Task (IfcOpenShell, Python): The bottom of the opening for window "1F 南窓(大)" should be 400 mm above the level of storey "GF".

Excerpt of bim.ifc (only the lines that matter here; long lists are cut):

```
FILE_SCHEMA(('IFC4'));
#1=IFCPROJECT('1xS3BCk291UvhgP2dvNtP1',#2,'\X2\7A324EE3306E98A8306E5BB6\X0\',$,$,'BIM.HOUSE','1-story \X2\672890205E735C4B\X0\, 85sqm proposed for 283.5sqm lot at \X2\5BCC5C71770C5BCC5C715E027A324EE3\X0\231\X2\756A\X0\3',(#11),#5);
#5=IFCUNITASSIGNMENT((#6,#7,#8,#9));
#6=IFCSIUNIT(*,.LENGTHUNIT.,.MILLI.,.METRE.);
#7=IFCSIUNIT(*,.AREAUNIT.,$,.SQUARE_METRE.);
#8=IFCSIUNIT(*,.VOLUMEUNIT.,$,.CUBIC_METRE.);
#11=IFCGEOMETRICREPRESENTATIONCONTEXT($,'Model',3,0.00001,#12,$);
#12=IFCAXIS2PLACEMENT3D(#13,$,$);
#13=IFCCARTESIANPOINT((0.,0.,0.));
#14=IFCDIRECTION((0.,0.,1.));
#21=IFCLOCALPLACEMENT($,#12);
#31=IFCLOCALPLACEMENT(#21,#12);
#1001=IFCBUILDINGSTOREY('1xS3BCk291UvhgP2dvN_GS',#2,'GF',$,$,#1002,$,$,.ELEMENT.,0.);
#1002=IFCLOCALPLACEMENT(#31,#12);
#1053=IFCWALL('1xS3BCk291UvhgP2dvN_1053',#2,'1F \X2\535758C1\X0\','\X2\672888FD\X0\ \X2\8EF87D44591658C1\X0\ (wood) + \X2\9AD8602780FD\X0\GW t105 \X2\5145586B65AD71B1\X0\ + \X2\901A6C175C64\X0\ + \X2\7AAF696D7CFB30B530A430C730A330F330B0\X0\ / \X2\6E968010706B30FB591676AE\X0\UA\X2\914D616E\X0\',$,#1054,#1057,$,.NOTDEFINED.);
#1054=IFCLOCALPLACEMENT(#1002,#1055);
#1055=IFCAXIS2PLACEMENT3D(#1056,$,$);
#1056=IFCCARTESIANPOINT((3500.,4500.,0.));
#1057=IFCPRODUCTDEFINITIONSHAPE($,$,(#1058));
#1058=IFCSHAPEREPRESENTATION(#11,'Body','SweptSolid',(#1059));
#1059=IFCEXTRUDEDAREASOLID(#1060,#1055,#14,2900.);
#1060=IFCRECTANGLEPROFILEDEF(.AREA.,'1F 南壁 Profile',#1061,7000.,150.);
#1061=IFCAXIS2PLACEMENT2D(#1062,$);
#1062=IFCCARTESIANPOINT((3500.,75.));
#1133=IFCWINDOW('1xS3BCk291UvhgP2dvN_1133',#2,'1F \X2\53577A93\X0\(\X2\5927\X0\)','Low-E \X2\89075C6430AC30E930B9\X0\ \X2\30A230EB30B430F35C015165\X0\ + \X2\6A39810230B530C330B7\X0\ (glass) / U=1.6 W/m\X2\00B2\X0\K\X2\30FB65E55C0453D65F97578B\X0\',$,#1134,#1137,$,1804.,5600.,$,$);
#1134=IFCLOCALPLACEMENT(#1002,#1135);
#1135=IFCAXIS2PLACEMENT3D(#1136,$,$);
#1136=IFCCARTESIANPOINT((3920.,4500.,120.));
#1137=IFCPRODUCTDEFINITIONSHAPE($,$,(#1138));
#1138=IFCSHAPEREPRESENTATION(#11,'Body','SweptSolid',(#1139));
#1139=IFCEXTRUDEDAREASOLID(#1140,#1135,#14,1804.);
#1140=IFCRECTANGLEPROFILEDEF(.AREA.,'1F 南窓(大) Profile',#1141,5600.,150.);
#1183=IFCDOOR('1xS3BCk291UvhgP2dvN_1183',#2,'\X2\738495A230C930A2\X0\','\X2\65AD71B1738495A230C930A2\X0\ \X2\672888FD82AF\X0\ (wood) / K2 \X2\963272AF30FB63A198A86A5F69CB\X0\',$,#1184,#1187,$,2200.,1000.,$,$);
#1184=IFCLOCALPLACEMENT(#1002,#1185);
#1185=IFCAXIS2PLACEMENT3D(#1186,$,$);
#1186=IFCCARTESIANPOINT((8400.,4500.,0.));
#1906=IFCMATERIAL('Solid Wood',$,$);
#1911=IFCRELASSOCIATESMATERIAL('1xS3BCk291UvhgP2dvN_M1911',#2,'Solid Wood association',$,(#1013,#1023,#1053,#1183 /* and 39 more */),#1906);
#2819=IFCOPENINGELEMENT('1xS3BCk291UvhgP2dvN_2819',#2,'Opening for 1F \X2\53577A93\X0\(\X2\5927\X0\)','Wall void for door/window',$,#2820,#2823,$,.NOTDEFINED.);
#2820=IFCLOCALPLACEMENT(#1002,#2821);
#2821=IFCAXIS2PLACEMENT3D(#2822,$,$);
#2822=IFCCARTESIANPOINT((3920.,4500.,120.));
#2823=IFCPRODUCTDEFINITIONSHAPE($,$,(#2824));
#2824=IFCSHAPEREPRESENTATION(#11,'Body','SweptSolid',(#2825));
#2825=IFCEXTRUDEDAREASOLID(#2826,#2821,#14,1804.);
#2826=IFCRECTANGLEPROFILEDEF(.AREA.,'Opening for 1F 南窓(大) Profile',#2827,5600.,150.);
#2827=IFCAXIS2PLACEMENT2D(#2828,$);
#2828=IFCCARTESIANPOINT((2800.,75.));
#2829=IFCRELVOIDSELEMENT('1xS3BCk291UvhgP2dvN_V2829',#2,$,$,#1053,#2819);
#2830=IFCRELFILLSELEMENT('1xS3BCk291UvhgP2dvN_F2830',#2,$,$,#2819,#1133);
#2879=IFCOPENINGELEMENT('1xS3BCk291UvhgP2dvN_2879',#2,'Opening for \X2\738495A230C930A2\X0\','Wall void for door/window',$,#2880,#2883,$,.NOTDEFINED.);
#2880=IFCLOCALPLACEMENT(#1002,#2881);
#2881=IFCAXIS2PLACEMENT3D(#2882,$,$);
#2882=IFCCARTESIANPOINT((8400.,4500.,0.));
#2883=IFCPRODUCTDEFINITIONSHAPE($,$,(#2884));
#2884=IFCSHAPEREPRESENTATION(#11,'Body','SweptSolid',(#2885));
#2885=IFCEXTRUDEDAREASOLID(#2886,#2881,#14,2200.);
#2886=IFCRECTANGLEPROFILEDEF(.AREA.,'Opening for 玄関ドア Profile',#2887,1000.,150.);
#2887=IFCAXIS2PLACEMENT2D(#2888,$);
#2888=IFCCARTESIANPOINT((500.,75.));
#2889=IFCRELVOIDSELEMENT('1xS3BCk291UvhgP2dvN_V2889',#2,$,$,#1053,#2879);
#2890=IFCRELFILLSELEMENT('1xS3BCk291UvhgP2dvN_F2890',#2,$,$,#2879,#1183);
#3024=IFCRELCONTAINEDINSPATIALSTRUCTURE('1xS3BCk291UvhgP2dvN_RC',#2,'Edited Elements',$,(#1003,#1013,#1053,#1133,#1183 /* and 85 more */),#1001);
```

```python
import numpy as np
import ifcopenshell
import ifcopenshell.api.geometry
import ifcopenshell.geom
import ifcopenshell.util.element
import ifcopenshell.util.placement
import ifcopenshell.util.shape
import ifcopenshell.util.unit

model = ifcopenshell.open("bim.ifc")
unit_scale = ifcopenshell.util.unit.calculate_unit_scale(model)

window = model.by_guid("1xS3BCk291UvhgP2dvN_1133")
opening = window.FillsVoids[0].RelatingOpeningElement
storey = ifcopenshell.util.element.get_container(window, ifc_class="IfcBuildingStorey")
level = ifcopenshell.util.placement.get_local_placement(storey.ObjectPlacement)[2, 3]

# The opening's origin need not be at the sill, so measure its lowest point.
shape = ifcopenshell.geom.create_shape(ifcopenshell.geom.settings(), opening)
bottom = ifcopenshell.util.shape.get_shape_bottom_elevation(shape, shape.geometry) / unit_scale
dz = level + 400.0 - bottom

shift = np.array([0.0, 0.0, dz])
# The window is not placed relative to its opening, so move both.
for product in (opening, window):
    matrix = ifcopenshell.util.placement.get_local_placement(product.ObjectPlacement)
    matrix[:3, 3] += shift
    ifcopenshell.api.geometry.edit_object_placement(model, product=product, matrix=matrix, is_si=False)

print(f"moved by {dz * unit_scale:+.3f} m")

model.write("bim-out.ifc")
```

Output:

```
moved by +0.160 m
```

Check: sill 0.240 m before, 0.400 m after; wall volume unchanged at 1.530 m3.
